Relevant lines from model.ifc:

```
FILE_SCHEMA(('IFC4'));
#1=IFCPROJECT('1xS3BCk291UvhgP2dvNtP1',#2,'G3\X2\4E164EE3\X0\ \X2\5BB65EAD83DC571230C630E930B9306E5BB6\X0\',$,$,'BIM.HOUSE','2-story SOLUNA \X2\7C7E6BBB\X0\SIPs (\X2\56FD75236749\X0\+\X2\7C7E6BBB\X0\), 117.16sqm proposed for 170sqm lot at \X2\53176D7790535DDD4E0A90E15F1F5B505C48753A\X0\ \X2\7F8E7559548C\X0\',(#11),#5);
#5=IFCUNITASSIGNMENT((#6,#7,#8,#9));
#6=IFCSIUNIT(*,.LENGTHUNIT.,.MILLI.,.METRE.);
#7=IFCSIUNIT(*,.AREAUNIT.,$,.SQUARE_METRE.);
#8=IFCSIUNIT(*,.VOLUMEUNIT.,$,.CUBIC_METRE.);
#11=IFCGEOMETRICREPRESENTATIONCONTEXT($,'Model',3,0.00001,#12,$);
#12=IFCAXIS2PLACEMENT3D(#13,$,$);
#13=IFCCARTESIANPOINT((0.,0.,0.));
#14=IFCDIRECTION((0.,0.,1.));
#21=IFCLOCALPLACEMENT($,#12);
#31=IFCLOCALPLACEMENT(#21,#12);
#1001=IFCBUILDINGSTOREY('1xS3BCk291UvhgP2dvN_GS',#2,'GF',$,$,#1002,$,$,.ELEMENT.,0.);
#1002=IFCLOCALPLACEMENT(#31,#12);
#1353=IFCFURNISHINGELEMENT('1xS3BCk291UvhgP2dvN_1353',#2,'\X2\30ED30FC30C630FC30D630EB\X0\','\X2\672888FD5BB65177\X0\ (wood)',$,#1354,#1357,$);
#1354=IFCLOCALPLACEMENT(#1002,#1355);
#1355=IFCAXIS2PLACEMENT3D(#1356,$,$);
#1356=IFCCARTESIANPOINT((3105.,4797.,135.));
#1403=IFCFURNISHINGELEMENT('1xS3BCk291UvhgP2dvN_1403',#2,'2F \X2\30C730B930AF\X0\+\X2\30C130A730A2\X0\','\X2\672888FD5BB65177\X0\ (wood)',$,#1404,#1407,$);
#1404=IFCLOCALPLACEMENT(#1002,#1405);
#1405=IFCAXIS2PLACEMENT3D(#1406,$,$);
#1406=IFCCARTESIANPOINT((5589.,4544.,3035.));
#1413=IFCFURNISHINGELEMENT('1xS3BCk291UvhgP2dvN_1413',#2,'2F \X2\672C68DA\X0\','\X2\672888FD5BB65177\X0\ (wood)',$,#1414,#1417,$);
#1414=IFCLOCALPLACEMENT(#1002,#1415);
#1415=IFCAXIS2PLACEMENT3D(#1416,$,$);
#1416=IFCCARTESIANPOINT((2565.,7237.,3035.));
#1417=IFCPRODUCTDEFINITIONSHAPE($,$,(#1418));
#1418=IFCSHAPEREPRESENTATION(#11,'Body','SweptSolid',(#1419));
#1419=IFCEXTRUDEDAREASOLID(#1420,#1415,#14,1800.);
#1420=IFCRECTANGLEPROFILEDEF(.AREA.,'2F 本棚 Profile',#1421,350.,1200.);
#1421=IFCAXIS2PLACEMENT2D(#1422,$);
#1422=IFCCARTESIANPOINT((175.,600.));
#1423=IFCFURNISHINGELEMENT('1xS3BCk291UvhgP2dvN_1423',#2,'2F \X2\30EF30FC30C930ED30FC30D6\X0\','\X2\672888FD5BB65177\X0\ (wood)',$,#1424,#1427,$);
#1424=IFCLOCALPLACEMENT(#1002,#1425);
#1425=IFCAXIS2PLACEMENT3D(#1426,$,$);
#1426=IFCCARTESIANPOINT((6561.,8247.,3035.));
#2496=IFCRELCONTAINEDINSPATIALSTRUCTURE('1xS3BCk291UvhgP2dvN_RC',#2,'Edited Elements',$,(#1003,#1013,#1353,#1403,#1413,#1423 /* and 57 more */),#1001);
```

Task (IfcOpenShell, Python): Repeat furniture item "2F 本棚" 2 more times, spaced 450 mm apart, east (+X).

```python
import numpy as np
import ifcopenshell
import ifcopenshell.api.geometry
import ifcopenshell.api.root
import ifcopenshell.util.element
import ifcopenshell.util.placement
import ifcopenshell.util.unit

model = ifcopenshell.open("model.ifc")
unit_scale = ifcopenshell.util.unit.calculate_unit_scale(model)


def reuse_history(source, copy):
    """copy_class also copies each property set's owner history, people and application; keep the originals."""
    for rel in copy.IsDefinedBy:
        if rel.is_a("IfcRelDefinesByProperties") and (history := rel.RelatingPropertyDefinition.OwnerHistory):
            rel.RelatingPropertyDefinition.OwnerHistory = source.OwnerHistory
            ifcopenshell.util.element.remove_deep2(model, history)


source = model.by_id(1413)
base = ifcopenshell.util.placement.get_local_placement(source.ObjectPlacement)
step = np.array([1.0, 0.0, 0.0]) * 0.45 / unit_scale

for i in range(1, 3):
    copy = ifcopenshell.api.root.copy_class(model, product=source)
    copy.Representation = ifcopenshell.util.element.copy_deep(
        model, source.Representation, exclude=["IfcGeometricRepresentationContext", "IfcRepresentationMap"]
    )
    reuse_history(source, copy)
    matrix = base.copy()
    matrix[:3, 3] += i * step
    print("added at", matrix[:3, 3].round(3) + 0.0)
    ifcopenshell.api.geometry.edit_object_placement(model, product=copy, matrix=matrix, is_si=False)

model.write("model_edited.ifc")
```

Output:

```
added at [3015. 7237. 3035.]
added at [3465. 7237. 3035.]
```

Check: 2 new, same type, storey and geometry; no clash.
